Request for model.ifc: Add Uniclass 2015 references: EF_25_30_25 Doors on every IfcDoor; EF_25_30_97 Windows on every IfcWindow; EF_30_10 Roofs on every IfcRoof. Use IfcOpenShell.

First a look at what the model holds.

```python
import ifcopenshell

model = ifcopenshell.open("model.ifc")
print(model.schema)
print("classifications:", [c.Name for c in model.by_type("IfcClassification")])
for ifc_class in ("IfcDoor", "IfcRoof", "IfcStair", "IfcWall", "IfcWindow"):
    print(ifc_class, len(model.by_type(ifc_class)))
```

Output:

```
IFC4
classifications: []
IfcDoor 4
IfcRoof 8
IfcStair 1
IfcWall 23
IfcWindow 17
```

```python
import ifcopenshell
import ifcopenshell.api.classification

model = ifcopenshell.open("model.ifc")

system = ifcopenshell.api.classification.add_classification(model, classification="Uniclass 2015")

codes = {
    "IfcDoor": ("EF_25_30_25", "Doors"),
    "IfcWindow": ("EF_25_30_97", "Windows"),
    "IfcRoof": ("EF_30_10", "Roofs"),
}
for ifc_class, (code, name) in codes.items():
    products = model.by_type(ifc_class)
    ifcopenshell.api.classification.add_reference(
        model, products=products, classification=system, identification=code, name=name
    )
    print(code, len(products))

model.write("model_rev.ifc")
```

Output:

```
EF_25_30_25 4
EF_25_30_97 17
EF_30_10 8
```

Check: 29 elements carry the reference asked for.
